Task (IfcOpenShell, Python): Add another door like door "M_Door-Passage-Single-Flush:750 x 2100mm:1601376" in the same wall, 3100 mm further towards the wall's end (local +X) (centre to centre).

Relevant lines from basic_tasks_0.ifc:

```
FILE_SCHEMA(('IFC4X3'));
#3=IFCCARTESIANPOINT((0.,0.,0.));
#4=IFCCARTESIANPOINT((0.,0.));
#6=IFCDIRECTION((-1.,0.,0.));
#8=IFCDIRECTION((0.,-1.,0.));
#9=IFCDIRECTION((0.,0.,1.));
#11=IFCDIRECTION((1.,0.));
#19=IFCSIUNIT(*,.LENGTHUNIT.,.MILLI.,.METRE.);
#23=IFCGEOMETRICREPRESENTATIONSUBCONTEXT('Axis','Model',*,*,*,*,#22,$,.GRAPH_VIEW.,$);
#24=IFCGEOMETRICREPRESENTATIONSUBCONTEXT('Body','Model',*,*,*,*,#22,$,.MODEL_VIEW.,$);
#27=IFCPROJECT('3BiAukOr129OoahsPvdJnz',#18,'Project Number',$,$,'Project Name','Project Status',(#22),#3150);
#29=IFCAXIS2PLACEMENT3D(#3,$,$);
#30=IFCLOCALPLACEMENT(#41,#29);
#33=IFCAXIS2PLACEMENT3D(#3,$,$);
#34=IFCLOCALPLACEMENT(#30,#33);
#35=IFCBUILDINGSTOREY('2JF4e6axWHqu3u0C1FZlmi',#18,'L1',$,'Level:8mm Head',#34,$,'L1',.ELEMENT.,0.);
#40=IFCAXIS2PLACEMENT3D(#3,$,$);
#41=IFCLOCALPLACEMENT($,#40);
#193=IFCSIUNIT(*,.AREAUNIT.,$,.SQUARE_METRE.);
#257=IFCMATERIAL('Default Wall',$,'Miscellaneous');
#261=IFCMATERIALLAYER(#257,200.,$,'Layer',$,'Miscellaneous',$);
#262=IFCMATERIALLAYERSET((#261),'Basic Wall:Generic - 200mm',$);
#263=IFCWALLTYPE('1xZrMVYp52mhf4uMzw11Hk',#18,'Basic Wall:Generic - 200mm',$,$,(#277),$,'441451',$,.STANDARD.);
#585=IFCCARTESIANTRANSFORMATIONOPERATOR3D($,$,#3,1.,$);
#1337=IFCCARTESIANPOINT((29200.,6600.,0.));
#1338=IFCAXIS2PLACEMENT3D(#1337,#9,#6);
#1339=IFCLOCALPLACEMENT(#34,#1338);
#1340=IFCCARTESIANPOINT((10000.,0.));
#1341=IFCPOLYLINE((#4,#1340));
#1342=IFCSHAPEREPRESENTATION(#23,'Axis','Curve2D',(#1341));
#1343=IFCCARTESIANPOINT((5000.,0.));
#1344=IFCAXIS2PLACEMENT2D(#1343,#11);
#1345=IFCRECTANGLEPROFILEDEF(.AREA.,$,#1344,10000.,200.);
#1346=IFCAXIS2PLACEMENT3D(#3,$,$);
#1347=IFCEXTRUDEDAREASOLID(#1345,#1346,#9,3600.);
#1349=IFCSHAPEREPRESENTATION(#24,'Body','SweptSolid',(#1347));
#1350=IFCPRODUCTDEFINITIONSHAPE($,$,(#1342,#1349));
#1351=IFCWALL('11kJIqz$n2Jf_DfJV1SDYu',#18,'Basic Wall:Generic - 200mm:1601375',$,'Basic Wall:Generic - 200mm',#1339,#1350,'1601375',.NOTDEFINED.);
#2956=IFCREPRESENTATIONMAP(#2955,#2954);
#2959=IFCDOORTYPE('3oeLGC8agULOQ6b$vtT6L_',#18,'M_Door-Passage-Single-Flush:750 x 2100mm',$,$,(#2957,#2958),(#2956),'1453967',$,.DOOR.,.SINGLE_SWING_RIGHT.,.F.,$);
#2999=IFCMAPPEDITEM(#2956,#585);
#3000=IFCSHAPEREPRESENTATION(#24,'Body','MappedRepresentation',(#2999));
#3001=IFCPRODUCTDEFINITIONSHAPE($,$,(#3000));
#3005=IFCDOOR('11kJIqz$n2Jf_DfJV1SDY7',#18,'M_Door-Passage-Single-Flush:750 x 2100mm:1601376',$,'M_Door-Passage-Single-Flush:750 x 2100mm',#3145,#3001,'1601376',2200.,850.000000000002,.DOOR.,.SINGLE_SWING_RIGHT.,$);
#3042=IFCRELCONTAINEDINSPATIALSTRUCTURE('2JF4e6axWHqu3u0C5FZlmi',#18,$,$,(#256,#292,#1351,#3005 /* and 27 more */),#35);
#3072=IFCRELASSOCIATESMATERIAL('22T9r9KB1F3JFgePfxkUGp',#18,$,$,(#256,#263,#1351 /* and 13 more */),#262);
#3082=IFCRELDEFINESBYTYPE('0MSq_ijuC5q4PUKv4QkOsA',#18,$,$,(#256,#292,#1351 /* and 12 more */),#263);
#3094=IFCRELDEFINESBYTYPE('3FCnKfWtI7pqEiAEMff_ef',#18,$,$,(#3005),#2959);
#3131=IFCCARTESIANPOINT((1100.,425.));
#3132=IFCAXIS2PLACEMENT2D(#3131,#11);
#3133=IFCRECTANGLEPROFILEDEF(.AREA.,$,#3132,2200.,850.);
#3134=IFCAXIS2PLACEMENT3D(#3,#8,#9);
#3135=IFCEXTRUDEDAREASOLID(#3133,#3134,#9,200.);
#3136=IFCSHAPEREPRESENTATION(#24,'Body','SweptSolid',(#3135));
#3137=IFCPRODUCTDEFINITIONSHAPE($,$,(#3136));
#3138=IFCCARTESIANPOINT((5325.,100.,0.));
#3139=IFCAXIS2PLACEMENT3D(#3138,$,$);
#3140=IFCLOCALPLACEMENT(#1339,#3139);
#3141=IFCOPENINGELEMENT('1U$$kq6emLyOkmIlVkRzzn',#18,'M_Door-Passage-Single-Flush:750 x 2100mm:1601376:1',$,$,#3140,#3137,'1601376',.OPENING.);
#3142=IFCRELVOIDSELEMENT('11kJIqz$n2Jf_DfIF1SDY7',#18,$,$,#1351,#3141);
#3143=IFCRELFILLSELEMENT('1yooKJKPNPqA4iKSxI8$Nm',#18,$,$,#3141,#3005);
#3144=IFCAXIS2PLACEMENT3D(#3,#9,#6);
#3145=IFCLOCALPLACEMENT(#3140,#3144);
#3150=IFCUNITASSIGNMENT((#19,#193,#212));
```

```python
import ifcopenshell
import ifcopenshell.api.feature
import ifcopenshell.api.geometry
import ifcopenshell.api.root
import ifcopenshell.geom
import ifcopenshell.util.element
import ifcopenshell.util.placement
import ifcopenshell.util.shape

model = ifcopenshell.open("basic_tasks_0.ifc")
settings = ifcopenshell.geom.settings()


def volume(element):
    """Net volume in cubic metres, openings subtracted."""
    shape = ifcopenshell.geom.create_shape(settings, element)
    return ifcopenshell.util.shape.get_volume(shape.geometry)


def reuse_history(source, copy):
    """copy_class also copies each property set's owner history, people and application; keep the originals."""
    for rel in copy.IsDefinedBy:
        if rel.is_a("IfcRelDefinesByProperties") and (history := rel.RelatingPropertyDefinition.OwnerHistory):
            rel.RelatingPropertyDefinition.OwnerHistory = source.OwnerHistory
            ifcopenshell.util.element.remove_deep2(model, history)


door = model.by_guid("11kJIqz$n2Jf_DfJV1SDY7")
opening = door.FillsVoids[0].RelatingOpeningElement
wall = opening.VoidsElements[0].RelatingBuildingElement
before = volume(wall)
shift = ifcopenshell.util.placement.get_local_placement(wall.ObjectPlacement)[:3, 0] * 3100.0

# copy_class copies the void relationship, type, container and properties, but no geometry.
new_opening = ifcopenshell.api.root.copy_class(model, product=opening)
new_opening.Representation = ifcopenshell.util.element.copy_deep(
    model, opening.Representation, exclude=["IfcGeometricRepresentationContext", "IfcRepresentationMap"]
)
new_opening.Name = "M_Door-Passage-Single-Flush:750 x 2100mm"
new_opening.Tag = None
new_door = ifcopenshell.api.root.copy_class(model, product=door)
new_door.Representation = ifcopenshell.util.element.copy_deep(
    model, door.Representation, exclude=["IfcGeometricRepresentationContext", "IfcRepresentationMap"]
)
new_door.Name = "M_Door-Passage-Single-Flush:750 x 2100mm"
new_door.Tag = None
reuse_history(door, new_door)
ifcopenshell.api.feature.add_filling(model, opening=new_opening, element=new_door)

for old, new in ((opening, new_opening), (door, new_door)):
    matrix = ifcopenshell.util.placement.get_local_placement(old.ObjectPlacement)
    matrix[:3, 3] += shift
    ifcopenshell.api.geometry.edit_object_placement(model, product=new, matrix=matrix, is_si=False)

after = volume(wall)

print(f"wall volume {before:.3f} -> {after:.3f} m3")

model.write("basic_tasks_0_v2.ifc")
```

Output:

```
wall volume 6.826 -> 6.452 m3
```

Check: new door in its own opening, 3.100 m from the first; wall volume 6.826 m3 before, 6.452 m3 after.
